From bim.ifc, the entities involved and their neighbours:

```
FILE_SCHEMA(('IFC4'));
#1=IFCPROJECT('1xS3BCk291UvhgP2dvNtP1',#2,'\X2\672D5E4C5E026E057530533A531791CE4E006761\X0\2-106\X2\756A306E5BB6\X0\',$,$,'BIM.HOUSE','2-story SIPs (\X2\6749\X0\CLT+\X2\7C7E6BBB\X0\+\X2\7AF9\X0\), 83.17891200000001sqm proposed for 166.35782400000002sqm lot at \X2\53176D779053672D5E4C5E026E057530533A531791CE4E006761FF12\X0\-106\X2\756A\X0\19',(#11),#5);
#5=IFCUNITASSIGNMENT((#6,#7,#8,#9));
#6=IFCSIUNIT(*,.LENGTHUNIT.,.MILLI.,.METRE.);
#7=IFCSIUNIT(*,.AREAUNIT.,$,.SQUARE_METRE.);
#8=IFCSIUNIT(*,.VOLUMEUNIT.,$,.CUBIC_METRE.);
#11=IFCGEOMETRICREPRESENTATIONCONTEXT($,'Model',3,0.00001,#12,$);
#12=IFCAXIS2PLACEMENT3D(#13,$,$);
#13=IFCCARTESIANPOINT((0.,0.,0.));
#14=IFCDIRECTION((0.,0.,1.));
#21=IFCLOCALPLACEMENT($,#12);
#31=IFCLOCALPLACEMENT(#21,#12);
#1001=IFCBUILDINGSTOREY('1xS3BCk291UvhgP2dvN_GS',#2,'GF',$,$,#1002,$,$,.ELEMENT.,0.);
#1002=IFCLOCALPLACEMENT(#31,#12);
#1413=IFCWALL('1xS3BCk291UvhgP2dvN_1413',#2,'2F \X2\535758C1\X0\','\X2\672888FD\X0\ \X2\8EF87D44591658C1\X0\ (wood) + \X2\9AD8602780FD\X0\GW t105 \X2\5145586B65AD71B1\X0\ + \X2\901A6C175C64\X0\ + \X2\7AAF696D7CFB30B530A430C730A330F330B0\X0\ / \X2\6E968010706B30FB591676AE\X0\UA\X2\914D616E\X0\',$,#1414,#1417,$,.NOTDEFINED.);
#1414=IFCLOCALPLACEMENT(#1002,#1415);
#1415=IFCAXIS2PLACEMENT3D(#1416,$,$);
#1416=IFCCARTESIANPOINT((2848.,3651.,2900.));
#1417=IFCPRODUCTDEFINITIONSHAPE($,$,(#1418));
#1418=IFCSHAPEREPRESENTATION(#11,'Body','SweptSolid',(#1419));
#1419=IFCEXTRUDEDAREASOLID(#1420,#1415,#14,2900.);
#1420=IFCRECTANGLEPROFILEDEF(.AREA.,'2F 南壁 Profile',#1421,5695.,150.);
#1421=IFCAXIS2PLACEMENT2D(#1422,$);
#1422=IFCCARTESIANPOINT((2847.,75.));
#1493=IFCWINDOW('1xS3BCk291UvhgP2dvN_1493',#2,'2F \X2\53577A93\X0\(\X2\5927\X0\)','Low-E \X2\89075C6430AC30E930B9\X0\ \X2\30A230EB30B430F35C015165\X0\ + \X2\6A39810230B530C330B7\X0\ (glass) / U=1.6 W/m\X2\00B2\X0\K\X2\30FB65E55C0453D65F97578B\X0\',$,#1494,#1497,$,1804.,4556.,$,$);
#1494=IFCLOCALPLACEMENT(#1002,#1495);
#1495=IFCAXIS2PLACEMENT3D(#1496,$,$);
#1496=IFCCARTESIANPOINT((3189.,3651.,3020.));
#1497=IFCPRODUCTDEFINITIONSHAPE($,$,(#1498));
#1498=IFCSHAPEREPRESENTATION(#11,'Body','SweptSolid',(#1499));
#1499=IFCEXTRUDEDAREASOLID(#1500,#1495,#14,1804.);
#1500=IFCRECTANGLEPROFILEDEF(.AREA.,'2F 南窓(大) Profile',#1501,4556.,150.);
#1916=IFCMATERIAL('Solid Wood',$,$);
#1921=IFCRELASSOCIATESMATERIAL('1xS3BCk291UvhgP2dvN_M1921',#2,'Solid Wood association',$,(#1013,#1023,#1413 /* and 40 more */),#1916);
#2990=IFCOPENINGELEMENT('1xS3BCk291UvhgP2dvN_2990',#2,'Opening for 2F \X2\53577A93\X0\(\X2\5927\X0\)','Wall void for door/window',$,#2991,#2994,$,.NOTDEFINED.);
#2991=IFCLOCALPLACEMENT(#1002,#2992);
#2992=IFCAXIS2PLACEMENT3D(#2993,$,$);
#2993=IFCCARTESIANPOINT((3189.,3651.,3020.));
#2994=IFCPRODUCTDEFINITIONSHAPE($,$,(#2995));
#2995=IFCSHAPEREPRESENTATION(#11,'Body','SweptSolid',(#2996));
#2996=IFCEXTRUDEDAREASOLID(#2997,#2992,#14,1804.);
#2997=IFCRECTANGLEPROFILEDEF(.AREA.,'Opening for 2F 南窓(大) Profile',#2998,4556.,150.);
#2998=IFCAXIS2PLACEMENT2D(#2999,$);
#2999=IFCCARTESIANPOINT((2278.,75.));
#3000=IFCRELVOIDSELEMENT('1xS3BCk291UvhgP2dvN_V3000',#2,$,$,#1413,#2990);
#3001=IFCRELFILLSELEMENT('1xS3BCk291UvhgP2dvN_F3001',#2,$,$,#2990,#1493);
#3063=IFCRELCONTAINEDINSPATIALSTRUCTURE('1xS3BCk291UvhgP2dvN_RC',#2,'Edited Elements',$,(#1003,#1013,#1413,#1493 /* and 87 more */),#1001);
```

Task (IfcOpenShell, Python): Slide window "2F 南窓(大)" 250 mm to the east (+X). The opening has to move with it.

```python
import ifcopenshell
import ifcopenshell.api.geometry
import ifcopenshell.util.placement
import ifcopenshell.util.unit

model = ifcopenshell.open("bim.ifc")
unit_scale = ifcopenshell.util.unit.calculate_unit_scale(model)

window = model.by_guid("1xS3BCk291UvhgP2dvN_1493")
opening = window.FillsVoids[0].RelatingOpeningElement
wall = opening.VoidsElements[0].RelatingBuildingElement

wall_matrix = ifcopenshell.util.placement.get_local_placement(wall.ObjectPlacement)
shift = wall_matrix[:3, 0] * 0.25 / unit_scale
before = ifcopenshell.util.placement.get_local_placement(window.ObjectPlacement)[:3, 3].copy()

# The window is not placed relative to its opening, so move both.
for product in (opening, window):
    matrix = ifcopenshell.util.placement.get_local_placement(product.ObjectPlacement)
    matrix[:3, 3] += shift
    ifcopenshell.api.geometry.edit_object_placement(model, product=product, matrix=matrix, is_si=False)

after = ifcopenshell.util.placement.get_local_placement(window.ObjectPlacement)[:3, 3]
print("window moved by", (after - before).round(3) + 0.0)

model.write("bim_rev.ifc")
```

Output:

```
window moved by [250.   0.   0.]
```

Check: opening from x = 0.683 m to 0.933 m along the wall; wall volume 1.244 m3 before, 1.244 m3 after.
